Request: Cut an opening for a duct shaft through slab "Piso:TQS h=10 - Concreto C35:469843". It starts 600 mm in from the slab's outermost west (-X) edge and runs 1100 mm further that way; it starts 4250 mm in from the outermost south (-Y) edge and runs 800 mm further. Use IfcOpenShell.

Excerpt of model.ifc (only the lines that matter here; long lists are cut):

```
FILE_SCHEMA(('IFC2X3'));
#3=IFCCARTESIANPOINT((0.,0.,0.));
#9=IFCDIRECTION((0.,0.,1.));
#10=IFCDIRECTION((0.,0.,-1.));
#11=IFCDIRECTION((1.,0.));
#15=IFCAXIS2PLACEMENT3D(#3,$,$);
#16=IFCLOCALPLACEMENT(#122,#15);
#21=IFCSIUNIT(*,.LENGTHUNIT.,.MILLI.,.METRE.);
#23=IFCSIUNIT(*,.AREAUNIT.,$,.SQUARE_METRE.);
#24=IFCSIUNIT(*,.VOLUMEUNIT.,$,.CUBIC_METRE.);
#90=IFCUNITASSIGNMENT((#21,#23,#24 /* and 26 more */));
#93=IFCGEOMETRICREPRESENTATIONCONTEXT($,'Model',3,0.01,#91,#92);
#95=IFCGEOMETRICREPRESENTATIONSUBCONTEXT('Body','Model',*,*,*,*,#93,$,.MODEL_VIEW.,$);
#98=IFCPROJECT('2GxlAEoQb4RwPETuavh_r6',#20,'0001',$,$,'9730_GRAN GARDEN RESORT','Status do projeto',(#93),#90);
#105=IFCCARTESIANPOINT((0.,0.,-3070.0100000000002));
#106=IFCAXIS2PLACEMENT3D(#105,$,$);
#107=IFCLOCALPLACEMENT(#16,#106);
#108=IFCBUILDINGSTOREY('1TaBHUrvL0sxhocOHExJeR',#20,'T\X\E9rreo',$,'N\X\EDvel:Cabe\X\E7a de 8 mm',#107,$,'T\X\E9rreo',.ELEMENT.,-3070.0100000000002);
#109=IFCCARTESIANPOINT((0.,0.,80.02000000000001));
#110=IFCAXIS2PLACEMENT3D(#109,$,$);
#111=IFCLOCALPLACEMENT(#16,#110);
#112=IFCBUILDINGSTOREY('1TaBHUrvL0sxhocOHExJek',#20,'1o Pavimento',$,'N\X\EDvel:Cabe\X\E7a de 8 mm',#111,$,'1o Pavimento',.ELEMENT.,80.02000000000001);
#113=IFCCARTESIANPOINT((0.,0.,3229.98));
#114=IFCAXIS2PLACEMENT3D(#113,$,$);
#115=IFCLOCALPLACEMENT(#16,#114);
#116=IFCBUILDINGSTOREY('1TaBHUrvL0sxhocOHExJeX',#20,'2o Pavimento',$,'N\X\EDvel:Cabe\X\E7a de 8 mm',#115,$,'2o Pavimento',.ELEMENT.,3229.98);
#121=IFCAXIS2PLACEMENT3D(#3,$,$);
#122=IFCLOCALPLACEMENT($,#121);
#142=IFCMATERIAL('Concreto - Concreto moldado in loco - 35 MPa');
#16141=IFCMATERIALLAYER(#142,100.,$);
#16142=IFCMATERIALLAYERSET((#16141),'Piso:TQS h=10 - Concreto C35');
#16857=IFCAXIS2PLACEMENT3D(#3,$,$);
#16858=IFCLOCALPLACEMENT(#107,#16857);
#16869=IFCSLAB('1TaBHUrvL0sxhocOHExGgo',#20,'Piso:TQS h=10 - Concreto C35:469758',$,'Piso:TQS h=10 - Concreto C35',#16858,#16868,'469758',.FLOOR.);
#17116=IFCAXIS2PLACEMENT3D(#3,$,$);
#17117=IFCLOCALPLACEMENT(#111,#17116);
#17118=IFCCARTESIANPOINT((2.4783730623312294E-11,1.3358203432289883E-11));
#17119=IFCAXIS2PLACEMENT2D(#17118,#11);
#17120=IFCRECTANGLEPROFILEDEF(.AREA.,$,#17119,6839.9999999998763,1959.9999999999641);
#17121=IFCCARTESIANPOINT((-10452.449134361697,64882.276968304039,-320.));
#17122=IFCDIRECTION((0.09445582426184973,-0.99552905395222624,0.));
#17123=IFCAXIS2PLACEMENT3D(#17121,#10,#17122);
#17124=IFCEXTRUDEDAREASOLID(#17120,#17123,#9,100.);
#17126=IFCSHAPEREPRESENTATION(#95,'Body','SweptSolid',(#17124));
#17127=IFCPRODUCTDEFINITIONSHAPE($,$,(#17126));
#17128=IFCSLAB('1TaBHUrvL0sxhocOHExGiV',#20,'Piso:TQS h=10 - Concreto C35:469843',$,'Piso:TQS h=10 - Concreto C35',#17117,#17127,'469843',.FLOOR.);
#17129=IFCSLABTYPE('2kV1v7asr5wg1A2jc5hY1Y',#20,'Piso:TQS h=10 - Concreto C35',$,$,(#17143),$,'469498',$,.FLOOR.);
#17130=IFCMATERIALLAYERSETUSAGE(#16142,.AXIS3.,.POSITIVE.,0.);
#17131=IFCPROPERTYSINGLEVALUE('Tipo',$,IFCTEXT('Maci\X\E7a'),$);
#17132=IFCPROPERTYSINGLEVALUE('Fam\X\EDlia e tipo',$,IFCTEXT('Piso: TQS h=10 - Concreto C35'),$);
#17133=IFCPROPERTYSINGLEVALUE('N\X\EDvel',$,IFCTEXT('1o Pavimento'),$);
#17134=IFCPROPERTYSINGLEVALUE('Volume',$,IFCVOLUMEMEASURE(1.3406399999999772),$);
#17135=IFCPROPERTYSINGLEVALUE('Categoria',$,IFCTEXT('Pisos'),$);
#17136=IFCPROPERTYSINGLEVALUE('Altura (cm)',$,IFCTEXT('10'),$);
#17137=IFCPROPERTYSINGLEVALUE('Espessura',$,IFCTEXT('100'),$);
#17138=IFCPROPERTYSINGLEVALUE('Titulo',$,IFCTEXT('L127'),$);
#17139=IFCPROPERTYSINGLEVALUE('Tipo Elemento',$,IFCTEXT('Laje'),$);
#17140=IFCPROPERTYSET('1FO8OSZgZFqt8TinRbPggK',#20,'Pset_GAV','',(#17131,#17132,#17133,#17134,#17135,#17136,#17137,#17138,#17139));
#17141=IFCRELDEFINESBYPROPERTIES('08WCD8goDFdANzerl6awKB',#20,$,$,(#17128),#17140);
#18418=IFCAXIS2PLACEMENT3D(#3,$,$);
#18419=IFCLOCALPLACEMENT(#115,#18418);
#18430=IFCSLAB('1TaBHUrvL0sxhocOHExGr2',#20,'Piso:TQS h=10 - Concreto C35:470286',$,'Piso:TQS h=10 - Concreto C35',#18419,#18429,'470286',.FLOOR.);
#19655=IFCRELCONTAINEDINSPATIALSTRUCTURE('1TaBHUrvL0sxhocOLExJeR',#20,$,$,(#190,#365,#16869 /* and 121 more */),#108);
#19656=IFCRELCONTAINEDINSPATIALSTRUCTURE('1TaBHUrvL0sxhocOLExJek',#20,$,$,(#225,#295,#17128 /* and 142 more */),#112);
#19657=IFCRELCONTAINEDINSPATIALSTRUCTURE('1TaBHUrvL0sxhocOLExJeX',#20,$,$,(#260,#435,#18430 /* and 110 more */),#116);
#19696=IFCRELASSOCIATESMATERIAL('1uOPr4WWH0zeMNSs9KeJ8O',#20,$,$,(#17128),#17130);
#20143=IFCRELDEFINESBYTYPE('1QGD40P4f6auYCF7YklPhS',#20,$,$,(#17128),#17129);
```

```python
import numpy as np
import ifcopenshell
import ifcopenshell.api.feature
import ifcopenshell.api.geometry
import ifcopenshell.api.pset
import ifcopenshell.api.root
import ifcopenshell.geom
import ifcopenshell.util.element
import ifcopenshell.util.placement
import ifcopenshell.util.representation
import ifcopenshell.util.shape
import ifcopenshell.util.unit

model = ifcopenshell.open("model.ifc")
unit_scale = ifcopenshell.util.unit.calculate_unit_scale(model)
volume_scale = ifcopenshell.util.unit.calculate_unit_scale(model, "VOLUMEUNIT")
settings = ifcopenshell.geom.settings()


def volume(element):
    """Net volume in cubic metres, openings subtracted."""
    shape = ifcopenshell.geom.create_shape(settings, element)
    return ifcopenshell.util.shape.get_volume(shape.geometry)


slab = model.by_guid("1TaBHUrvL0sxhocOHExGiV")
before = volume(slab)

# Extent in the slab's own axes, in metres. The edges named are its -X and -Y sides.
slab_shape = ifcopenshell.geom.create_shape(settings, slab)
vertices = ifcopenshell.util.shape.get_vertices(slab_shape.geometry)
x_min, y_min, bottom = vertices.min(axis=0)
top = vertices[:, 2].max()

opening = ifcopenshell.api.root.create_entity(model, ifc_class="IfcOpeningElement", name="Duct shaft opening")
context = ifcopenshell.util.representation.get_context(model, "Model", "Body", "MODEL_VIEW")
width, depth = 1.1, 0.8
outline = [(0.0, 0.0), (width, 0.0), (width, depth), (0.0, depth), (0.0, 0.0)]
# Overshoot both faces by 50 mm so the cut is clean.
shape = ifcopenshell.api.geometry.add_slab_representation(
    model, context=context, depth=top - bottom + 0.1, polyline=outline
)
ifcopenshell.api.geometry.assign_representation(model, product=opening, representation=shape)

matrix = ifcopenshell.util.placement.get_local_placement(slab.ObjectPlacement)
matrix[:, 3] = matrix @ np.append(np.array([x_min + 0.6, y_min + 4.25, bottom - 0.05]) / unit_scale, 1.0)
ifcopenshell.api.geometry.edit_object_placement(model, product=opening, matrix=matrix, is_si=False)
ifcopenshell.api.feature.add_feature(model, feature=opening, element=slab)

after = volume(slab)

# Update the slab's stored quantities.
pset = model.by_id(ifcopenshell.util.element.get_pset(slab, "Pset_GAV", should_inherit=False)["id"])
ifcopenshell.api.pset.edit_pset(model, pset=pset, properties={
    "Volume": model.create_entity("IfcVolumeMeasure", after / volume_scale),
})

print(f"slab volume {before:.3f} -> {after:.3f} m3")

model.write("model_updated.ifc")
```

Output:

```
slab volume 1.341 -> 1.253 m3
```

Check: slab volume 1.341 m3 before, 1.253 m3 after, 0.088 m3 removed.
